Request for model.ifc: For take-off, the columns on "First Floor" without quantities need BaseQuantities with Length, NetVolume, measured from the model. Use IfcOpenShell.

First a look at what the model holds.

```python
import ifcopenshell
import ifcopenshell.util.element
import ifcopenshell.util.unit

model = ifcopenshell.open("model.ifc")
print(model.schema)
for unit_type in ("LENGTHUNIT", "AREAUNIT", "VOLUMEUNIT"):
    print(unit_type, ifcopenshell.util.unit.calculate_unit_scale(model, unit_type))
storey = next(s for s in model.by_type("IfcBuildingStorey") if s.Name == "First Floor")
columns = [e for e in ifcopenshell.util.element.get_decomposition(storey) if e.is_a("IfcColumn")]
for e in sorted(columns, key=lambda e: e.id()):
    print(e.id(), e.is_a(), e.Name, list(ifcopenshell.util.element.get_psets(e, qtos_only=True)), sep=" | ")
```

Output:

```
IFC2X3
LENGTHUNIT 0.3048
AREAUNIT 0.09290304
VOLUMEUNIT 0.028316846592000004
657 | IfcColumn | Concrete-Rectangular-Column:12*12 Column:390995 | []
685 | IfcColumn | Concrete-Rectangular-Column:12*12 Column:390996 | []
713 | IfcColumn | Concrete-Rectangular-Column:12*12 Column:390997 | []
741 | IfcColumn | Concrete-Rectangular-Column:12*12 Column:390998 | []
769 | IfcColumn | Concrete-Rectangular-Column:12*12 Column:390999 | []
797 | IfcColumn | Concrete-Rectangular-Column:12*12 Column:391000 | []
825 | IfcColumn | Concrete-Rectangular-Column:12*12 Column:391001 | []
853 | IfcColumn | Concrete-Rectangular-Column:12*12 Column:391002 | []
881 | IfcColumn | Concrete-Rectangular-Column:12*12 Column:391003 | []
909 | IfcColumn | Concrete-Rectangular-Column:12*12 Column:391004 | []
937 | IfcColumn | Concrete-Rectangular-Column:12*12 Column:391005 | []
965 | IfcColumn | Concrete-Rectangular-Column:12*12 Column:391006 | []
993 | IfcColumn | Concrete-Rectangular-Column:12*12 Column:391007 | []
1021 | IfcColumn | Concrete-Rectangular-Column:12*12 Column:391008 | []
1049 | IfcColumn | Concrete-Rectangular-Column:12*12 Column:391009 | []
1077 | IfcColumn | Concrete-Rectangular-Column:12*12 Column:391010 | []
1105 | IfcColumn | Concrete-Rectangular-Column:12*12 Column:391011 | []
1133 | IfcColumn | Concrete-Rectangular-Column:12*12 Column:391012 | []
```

```python
import ifcopenshell
import ifcopenshell.api.pset
import ifcopenshell.geom
import ifcopenshell.util.element
import ifcopenshell.util.shape
import ifcopenshell.util.unit

model = ifcopenshell.open("model.ifc")
unit_scale = ifcopenshell.util.unit.calculate_unit_scale(model)
volume_scale = ifcopenshell.util.unit.calculate_unit_scale(model, "VOLUMEUNIT")
settings = ifcopenshell.geom.settings()

storey = next(s for s in model.by_type("IfcBuildingStorey") if s.Name == "First Floor")
columns = [e for e in ifcopenshell.util.element.get_decomposition(storey) if e.is_a("IfcColumn")]

for e in sorted(columns, key=lambda e: e.id()):
    if ifcopenshell.util.element.get_psets(e, qtos_only=True, should_inherit=False):
        continue
    # Geometry comes back in metres, in the element's own axes.
    shape = ifcopenshell.geom.create_shape(settings, e)
    values = {
        "Length": ifcopenshell.util.shape.get_z(shape.geometry) / unit_scale,
        "NetVolume": ifcopenshell.util.shape.get_volume(shape.geometry) / volume_scale,
    }
    qto = ifcopenshell.api.pset.add_qto(model, product=e, name="BaseQuantities")
    ifcopenshell.api.pset.edit_qto(model, qto=qto, properties=values)
    print(e.id(), {k: round(v, 3) for k, v in values.items()})

model.write("model_updated.ifc")
```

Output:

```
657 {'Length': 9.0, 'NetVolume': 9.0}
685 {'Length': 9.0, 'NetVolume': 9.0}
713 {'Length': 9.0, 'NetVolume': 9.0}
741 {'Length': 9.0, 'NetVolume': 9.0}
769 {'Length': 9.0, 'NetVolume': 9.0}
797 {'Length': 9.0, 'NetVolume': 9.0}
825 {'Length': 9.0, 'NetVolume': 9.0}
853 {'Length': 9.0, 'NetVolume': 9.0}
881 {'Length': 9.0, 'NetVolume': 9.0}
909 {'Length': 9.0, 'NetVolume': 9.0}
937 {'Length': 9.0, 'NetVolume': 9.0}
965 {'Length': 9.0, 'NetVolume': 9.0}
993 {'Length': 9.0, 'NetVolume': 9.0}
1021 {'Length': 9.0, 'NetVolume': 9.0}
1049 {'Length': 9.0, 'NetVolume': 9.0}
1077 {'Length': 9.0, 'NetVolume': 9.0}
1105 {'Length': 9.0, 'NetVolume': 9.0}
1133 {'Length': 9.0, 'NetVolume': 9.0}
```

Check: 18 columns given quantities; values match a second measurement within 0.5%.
